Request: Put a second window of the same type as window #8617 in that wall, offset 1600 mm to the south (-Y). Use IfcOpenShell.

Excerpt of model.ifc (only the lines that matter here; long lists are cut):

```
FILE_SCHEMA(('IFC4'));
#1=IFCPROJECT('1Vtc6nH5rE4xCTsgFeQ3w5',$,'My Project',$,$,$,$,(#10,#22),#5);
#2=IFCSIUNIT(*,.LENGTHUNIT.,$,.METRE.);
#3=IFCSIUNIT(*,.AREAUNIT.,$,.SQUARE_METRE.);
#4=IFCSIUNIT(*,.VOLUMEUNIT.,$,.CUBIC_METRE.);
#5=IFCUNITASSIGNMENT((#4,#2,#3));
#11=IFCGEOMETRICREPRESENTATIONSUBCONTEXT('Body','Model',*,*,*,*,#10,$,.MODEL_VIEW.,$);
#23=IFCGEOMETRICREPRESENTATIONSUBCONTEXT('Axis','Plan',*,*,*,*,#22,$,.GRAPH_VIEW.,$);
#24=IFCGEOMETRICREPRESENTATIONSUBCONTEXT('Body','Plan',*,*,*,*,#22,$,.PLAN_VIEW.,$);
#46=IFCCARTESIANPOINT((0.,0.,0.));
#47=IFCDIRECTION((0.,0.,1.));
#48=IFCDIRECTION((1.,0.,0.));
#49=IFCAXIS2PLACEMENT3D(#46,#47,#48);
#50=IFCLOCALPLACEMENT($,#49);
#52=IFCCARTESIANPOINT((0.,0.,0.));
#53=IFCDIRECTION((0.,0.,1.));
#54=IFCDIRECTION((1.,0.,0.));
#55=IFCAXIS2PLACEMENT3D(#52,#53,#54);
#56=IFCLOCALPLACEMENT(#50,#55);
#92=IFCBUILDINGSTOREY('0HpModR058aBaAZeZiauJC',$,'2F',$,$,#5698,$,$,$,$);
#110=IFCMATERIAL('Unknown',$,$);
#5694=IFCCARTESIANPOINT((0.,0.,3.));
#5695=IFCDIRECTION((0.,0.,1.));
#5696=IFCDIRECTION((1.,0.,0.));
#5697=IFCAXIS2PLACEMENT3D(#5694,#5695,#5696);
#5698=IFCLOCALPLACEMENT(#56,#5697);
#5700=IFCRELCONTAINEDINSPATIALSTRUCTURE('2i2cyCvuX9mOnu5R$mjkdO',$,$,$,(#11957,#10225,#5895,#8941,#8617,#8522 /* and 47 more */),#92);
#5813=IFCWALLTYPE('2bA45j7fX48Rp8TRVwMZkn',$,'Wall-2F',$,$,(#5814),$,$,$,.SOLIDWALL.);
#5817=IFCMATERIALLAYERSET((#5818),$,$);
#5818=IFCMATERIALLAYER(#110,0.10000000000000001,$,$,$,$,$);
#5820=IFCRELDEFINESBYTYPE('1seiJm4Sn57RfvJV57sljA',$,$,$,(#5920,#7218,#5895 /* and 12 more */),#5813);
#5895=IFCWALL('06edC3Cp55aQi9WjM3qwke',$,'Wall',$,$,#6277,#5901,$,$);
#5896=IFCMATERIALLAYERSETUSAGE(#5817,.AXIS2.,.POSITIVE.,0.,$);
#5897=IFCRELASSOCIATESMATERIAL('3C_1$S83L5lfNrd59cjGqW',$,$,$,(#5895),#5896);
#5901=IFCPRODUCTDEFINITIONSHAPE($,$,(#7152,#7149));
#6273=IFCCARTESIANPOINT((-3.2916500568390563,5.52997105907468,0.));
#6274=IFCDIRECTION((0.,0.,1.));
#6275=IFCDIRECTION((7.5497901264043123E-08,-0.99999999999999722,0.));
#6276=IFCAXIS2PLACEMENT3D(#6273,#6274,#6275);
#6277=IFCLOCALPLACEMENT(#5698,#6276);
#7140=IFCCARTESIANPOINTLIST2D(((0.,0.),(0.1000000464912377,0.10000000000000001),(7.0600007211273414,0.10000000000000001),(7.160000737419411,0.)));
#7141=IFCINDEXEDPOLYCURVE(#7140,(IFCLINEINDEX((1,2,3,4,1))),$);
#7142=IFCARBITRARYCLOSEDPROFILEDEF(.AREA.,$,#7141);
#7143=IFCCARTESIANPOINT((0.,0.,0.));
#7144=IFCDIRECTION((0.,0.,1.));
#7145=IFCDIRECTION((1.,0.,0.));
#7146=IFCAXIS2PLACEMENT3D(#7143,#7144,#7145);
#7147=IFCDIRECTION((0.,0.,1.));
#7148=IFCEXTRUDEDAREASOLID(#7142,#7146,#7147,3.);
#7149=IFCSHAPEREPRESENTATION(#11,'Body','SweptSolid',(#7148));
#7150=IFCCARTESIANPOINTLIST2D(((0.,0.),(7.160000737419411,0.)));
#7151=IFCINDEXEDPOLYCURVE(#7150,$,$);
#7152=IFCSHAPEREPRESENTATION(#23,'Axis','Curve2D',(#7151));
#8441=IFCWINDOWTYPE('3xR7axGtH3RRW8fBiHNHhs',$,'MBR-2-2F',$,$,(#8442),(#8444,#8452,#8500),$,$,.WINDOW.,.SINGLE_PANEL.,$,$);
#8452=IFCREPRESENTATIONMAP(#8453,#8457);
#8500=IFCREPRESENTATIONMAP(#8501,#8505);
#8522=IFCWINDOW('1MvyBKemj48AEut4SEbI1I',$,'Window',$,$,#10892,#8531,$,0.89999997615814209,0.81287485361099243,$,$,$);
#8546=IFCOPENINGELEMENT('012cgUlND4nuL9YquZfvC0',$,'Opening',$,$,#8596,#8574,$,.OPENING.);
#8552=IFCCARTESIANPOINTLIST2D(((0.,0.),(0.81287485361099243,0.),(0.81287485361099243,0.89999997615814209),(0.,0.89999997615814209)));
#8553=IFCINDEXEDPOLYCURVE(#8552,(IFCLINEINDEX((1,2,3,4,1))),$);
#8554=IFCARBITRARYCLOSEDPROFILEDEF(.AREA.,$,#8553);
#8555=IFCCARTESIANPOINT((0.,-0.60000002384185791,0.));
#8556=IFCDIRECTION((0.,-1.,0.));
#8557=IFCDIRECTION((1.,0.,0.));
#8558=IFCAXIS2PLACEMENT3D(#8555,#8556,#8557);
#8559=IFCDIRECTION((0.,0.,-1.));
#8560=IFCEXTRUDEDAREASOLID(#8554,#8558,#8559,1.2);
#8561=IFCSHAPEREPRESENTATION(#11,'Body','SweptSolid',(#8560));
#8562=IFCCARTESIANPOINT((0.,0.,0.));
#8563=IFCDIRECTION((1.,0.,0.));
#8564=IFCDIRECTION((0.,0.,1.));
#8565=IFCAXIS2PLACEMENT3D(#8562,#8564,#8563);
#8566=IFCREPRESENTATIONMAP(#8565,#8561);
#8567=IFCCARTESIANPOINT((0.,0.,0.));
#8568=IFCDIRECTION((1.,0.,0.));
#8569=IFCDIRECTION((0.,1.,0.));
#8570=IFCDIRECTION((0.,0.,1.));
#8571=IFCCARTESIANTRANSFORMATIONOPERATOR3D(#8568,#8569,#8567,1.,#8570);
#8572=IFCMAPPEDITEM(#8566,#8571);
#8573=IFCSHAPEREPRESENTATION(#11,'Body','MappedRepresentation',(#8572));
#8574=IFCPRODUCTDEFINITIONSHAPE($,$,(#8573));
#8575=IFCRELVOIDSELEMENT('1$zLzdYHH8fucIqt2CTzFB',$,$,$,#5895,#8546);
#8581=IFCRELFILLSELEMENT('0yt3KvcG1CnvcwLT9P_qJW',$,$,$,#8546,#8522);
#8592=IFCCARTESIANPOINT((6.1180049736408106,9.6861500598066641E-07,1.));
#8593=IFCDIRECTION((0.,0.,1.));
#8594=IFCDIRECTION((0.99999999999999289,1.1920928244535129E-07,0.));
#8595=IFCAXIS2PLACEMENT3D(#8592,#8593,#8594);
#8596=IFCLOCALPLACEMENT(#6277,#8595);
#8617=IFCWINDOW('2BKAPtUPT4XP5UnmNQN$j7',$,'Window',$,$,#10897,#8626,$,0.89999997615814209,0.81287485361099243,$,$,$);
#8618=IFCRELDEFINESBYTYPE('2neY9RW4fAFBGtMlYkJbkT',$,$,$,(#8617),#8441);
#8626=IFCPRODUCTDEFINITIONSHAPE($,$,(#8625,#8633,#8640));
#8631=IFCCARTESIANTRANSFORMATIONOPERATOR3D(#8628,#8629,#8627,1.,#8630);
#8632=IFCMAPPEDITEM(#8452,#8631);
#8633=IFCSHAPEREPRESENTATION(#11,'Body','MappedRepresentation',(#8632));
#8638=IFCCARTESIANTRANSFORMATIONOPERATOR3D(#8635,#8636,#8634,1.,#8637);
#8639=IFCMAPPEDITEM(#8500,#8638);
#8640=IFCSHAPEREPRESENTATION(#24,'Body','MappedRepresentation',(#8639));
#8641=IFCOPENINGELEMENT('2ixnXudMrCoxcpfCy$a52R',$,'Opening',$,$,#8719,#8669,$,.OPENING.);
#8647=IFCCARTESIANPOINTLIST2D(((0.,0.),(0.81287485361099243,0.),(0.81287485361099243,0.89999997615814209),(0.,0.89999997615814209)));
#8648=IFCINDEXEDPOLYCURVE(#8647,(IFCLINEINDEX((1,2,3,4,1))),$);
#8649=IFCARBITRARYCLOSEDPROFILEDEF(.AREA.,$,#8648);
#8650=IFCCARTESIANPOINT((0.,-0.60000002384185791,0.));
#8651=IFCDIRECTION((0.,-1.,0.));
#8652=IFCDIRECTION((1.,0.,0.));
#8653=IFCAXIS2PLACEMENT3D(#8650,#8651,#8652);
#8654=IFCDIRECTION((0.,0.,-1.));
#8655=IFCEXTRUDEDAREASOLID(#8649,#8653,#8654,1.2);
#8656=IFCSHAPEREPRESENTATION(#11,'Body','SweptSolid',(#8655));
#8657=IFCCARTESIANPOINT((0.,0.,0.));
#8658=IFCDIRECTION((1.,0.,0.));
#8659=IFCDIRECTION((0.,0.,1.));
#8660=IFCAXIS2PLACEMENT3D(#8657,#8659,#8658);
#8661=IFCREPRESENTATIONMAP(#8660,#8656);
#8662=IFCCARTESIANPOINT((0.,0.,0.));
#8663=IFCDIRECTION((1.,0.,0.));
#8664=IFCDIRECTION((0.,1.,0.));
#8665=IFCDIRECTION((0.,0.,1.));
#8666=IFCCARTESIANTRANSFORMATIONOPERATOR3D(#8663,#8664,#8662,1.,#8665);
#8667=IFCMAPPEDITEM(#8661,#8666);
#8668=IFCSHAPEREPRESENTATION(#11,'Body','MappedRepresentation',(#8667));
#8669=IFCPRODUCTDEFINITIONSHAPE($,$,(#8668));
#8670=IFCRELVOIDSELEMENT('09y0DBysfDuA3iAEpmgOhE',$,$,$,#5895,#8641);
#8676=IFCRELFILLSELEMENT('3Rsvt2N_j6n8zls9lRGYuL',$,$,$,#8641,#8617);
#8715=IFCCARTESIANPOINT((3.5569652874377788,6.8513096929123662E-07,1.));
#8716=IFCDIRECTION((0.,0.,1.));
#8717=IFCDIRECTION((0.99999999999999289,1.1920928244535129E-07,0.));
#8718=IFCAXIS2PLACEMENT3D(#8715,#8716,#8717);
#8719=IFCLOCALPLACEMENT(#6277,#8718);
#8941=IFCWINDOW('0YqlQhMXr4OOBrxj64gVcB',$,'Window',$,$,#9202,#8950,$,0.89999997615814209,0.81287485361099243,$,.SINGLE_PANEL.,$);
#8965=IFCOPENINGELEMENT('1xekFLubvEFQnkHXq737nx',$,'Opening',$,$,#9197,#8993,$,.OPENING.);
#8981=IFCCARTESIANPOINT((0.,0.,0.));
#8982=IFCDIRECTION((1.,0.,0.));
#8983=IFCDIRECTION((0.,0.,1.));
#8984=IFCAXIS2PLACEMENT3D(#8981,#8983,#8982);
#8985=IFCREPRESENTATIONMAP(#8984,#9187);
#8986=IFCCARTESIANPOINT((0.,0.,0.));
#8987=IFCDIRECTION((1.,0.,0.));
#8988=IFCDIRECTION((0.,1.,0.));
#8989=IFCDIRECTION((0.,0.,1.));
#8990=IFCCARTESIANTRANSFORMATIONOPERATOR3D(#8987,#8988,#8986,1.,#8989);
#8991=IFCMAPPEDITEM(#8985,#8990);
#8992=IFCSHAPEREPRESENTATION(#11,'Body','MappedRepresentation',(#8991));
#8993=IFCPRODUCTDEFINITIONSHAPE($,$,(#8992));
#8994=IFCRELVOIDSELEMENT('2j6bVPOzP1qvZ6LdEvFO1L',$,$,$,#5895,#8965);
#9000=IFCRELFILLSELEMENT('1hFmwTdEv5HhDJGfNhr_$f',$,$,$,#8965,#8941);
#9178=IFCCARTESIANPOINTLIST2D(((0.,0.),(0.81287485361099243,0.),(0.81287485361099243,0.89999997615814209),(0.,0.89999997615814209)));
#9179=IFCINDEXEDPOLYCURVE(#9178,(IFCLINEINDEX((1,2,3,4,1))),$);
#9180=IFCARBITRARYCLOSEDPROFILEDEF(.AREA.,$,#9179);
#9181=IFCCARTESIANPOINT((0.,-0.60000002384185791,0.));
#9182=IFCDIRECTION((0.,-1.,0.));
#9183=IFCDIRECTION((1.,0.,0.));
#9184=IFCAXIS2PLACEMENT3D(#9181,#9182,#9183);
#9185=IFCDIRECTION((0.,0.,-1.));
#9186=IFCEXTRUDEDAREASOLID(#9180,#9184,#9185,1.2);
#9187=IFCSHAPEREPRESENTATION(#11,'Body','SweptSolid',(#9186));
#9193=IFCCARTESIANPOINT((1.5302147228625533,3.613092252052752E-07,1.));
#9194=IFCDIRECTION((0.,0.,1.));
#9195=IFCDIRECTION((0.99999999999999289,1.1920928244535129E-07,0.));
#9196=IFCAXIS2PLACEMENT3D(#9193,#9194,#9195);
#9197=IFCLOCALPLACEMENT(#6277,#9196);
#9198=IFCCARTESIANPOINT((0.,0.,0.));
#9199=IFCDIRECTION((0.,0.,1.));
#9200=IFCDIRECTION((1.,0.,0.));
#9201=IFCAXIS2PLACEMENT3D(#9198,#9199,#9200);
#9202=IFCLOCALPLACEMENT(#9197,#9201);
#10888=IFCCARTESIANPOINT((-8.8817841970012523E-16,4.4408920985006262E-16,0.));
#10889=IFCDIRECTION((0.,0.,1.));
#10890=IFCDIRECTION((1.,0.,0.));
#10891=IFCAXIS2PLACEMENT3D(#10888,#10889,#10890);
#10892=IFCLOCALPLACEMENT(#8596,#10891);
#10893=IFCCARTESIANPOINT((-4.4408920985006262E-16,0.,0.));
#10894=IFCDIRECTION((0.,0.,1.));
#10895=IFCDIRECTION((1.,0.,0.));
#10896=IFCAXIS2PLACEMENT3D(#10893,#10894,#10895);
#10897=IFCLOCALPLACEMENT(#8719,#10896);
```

```python
import ifcopenshell
import ifcopenshell.api.feature
import ifcopenshell.api.geometry
import ifcopenshell.api.root
import ifcopenshell.geom
import ifcopenshell.util.element
import ifcopenshell.util.placement
import ifcopenshell.util.shape
import ifcopenshell.util.unit

model = ifcopenshell.open("model.ifc")
unit_scale = ifcopenshell.util.unit.calculate_unit_scale(model)
settings = ifcopenshell.geom.settings()


def volume(element):
    """Net volume in cubic metres, openings subtracted."""
    shape = ifcopenshell.geom.create_shape(settings, element)
    return ifcopenshell.util.shape.get_volume(shape.geometry)


window = model.by_guid("2BKAPtUPT4XP5UnmNQN$j7")
opening = window.FillsVoids[0].RelatingOpeningElement
wall = opening.VoidsElements[0].RelatingBuildingElement
before = volume(wall)
shift = ifcopenshell.util.placement.get_local_placement(wall.ObjectPlacement)[:3, 0] * 1.6 / unit_scale

# copy_class copies the void relationship, type, container and properties, but no geometry.
new_opening = ifcopenshell.api.root.copy_class(model, product=opening)
new_opening.Representation = ifcopenshell.util.element.copy_deep(
    model, opening.Representation, exclude=["IfcGeometricRepresentationContext", "IfcRepresentationMap"]
)
new_window = ifcopenshell.api.root.copy_class(model, product=window)
new_window.Representation = ifcopenshell.util.element.copy_deep(
    model, window.Representation, exclude=["IfcGeometricRepresentationContext", "IfcRepresentationMap"]
)
ifcopenshell.api.feature.add_filling(model, opening=new_opening, element=new_window)

for old, new in ((opening, new_opening), (window, new_window)):
    matrix = ifcopenshell.util.placement.get_local_placement(old.ObjectPlacement)
    matrix[:3, 3] += shift
    ifcopenshell.api.geometry.edit_object_placement(model, product=new, matrix=matrix, is_si=False)

after = volume(wall)

print(f"wall volume {before:.3f} -> {after:.3f} m3")

model.write("model_rev.ifc")
```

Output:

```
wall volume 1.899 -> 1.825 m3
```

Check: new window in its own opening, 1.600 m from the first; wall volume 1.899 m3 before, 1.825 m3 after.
